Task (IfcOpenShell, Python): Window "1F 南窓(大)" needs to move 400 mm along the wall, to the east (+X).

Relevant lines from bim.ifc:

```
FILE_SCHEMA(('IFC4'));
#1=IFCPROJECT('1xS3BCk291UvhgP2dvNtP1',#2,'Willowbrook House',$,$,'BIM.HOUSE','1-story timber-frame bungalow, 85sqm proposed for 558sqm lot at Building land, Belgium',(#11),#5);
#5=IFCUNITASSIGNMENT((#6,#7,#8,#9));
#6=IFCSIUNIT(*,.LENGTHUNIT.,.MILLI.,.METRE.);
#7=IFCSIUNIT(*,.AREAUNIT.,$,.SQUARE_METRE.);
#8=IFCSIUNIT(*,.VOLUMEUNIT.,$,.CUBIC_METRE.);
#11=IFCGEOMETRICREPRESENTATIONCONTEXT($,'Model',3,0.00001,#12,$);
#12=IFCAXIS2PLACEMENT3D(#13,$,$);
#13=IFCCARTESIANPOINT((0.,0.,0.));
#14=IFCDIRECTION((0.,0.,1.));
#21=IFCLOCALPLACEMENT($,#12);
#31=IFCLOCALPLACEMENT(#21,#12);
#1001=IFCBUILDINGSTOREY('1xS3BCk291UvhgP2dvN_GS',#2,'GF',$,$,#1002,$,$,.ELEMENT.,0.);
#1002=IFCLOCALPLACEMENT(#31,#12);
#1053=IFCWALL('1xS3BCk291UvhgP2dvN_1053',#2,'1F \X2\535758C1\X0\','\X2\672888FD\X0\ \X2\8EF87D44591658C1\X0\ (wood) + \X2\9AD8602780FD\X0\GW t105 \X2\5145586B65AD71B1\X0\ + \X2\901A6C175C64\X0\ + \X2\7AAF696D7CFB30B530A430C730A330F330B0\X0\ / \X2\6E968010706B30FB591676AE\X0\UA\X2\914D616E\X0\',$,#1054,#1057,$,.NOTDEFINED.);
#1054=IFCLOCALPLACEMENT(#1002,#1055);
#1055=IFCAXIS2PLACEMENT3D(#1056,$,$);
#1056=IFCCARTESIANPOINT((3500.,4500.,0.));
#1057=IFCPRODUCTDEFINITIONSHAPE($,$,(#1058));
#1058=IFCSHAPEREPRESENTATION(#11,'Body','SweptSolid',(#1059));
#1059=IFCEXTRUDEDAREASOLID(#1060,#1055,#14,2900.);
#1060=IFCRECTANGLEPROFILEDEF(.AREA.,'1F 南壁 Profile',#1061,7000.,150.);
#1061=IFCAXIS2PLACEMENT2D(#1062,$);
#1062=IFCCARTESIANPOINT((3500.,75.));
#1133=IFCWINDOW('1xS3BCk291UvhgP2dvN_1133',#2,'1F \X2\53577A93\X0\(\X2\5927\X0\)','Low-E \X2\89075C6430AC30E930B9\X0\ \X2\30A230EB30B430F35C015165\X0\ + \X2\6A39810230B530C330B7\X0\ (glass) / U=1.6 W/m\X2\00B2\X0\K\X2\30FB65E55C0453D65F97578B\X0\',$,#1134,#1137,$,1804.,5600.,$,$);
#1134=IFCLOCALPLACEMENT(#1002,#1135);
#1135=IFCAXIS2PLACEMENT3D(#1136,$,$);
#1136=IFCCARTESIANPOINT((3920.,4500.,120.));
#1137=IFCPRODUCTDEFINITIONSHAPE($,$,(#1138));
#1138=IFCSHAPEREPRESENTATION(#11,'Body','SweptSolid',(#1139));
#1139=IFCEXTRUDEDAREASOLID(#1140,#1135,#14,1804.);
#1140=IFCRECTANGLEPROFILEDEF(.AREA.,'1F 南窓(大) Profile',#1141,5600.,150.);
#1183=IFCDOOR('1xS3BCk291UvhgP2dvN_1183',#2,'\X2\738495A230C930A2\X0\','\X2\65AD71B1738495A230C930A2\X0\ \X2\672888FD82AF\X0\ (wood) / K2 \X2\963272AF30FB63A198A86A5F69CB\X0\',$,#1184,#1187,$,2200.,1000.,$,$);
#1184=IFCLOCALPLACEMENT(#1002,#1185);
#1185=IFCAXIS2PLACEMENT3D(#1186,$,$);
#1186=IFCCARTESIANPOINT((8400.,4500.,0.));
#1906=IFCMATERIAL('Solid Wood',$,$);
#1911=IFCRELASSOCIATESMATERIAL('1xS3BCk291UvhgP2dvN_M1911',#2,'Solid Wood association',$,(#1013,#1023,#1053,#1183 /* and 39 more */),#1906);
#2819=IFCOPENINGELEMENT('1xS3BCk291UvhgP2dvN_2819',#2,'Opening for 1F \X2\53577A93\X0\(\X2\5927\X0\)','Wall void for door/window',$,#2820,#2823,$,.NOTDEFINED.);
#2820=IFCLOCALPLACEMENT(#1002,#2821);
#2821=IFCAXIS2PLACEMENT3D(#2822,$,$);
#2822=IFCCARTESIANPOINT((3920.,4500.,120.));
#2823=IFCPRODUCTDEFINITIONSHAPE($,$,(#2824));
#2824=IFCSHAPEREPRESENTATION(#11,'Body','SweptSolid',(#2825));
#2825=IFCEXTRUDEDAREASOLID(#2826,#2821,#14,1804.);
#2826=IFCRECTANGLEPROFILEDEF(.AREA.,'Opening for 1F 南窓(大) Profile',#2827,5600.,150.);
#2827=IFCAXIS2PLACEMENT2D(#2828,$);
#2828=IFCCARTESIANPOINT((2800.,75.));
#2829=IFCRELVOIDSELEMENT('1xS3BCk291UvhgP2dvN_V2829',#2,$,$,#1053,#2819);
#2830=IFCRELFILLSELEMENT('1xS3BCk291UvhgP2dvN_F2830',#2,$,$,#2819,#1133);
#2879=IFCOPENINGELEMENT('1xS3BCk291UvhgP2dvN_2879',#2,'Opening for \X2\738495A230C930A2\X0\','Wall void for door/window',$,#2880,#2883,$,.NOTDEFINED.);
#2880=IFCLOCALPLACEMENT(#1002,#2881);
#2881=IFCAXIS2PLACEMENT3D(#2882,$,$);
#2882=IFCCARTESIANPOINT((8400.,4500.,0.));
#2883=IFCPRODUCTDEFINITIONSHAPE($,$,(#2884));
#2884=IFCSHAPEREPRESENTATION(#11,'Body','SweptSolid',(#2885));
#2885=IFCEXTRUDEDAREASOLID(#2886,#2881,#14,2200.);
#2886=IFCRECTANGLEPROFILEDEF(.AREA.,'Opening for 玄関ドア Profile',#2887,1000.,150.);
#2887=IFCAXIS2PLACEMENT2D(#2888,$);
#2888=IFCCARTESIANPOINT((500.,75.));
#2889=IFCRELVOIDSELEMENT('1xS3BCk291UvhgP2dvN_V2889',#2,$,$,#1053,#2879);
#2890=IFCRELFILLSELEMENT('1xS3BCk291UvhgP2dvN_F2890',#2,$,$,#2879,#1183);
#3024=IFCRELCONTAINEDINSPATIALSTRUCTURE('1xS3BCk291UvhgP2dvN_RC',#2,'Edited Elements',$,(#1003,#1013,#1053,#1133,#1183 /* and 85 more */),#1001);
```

```python
import ifcopenshell
import ifcopenshell.api.geometry
import ifcopenshell.util.placement
import ifcopenshell.util.unit

model = ifcopenshell.open("bim.ifc")
unit_scale = ifcopenshell.util.unit.calculate_unit_scale(model)

window = model.by_id(1133)
opening = window.FillsVoids[0].RelatingOpeningElement
wall = opening.VoidsElements[0].RelatingBuildingElement

wall_matrix = ifcopenshell.util.placement.get_local_placement(wall.ObjectPlacement)
shift = wall_matrix[:3, 0] * 0.4 / unit_scale
before = ifcopenshell.util.placement.get_local_placement(window.ObjectPlacement)[:3, 3].copy()

# The window is not placed relative to its opening, so move both.
for product in (opening, window):
    matrix = ifcopenshell.util.placement.get_local_placement(product.ObjectPlacement)
    matrix[:3, 3] += shift
    ifcopenshell.api.geometry.edit_object_placement(model, product=product, matrix=matrix, is_si=False)

after = ifcopenshell.util.placement.get_local_placement(window.ObjectPlacement)[:3, 3]
print("window moved by", (after - before).round(3) + 0.0)

model.write("bim-out.ifc")
```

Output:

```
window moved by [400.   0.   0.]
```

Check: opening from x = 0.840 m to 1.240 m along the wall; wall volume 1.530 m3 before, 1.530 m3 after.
